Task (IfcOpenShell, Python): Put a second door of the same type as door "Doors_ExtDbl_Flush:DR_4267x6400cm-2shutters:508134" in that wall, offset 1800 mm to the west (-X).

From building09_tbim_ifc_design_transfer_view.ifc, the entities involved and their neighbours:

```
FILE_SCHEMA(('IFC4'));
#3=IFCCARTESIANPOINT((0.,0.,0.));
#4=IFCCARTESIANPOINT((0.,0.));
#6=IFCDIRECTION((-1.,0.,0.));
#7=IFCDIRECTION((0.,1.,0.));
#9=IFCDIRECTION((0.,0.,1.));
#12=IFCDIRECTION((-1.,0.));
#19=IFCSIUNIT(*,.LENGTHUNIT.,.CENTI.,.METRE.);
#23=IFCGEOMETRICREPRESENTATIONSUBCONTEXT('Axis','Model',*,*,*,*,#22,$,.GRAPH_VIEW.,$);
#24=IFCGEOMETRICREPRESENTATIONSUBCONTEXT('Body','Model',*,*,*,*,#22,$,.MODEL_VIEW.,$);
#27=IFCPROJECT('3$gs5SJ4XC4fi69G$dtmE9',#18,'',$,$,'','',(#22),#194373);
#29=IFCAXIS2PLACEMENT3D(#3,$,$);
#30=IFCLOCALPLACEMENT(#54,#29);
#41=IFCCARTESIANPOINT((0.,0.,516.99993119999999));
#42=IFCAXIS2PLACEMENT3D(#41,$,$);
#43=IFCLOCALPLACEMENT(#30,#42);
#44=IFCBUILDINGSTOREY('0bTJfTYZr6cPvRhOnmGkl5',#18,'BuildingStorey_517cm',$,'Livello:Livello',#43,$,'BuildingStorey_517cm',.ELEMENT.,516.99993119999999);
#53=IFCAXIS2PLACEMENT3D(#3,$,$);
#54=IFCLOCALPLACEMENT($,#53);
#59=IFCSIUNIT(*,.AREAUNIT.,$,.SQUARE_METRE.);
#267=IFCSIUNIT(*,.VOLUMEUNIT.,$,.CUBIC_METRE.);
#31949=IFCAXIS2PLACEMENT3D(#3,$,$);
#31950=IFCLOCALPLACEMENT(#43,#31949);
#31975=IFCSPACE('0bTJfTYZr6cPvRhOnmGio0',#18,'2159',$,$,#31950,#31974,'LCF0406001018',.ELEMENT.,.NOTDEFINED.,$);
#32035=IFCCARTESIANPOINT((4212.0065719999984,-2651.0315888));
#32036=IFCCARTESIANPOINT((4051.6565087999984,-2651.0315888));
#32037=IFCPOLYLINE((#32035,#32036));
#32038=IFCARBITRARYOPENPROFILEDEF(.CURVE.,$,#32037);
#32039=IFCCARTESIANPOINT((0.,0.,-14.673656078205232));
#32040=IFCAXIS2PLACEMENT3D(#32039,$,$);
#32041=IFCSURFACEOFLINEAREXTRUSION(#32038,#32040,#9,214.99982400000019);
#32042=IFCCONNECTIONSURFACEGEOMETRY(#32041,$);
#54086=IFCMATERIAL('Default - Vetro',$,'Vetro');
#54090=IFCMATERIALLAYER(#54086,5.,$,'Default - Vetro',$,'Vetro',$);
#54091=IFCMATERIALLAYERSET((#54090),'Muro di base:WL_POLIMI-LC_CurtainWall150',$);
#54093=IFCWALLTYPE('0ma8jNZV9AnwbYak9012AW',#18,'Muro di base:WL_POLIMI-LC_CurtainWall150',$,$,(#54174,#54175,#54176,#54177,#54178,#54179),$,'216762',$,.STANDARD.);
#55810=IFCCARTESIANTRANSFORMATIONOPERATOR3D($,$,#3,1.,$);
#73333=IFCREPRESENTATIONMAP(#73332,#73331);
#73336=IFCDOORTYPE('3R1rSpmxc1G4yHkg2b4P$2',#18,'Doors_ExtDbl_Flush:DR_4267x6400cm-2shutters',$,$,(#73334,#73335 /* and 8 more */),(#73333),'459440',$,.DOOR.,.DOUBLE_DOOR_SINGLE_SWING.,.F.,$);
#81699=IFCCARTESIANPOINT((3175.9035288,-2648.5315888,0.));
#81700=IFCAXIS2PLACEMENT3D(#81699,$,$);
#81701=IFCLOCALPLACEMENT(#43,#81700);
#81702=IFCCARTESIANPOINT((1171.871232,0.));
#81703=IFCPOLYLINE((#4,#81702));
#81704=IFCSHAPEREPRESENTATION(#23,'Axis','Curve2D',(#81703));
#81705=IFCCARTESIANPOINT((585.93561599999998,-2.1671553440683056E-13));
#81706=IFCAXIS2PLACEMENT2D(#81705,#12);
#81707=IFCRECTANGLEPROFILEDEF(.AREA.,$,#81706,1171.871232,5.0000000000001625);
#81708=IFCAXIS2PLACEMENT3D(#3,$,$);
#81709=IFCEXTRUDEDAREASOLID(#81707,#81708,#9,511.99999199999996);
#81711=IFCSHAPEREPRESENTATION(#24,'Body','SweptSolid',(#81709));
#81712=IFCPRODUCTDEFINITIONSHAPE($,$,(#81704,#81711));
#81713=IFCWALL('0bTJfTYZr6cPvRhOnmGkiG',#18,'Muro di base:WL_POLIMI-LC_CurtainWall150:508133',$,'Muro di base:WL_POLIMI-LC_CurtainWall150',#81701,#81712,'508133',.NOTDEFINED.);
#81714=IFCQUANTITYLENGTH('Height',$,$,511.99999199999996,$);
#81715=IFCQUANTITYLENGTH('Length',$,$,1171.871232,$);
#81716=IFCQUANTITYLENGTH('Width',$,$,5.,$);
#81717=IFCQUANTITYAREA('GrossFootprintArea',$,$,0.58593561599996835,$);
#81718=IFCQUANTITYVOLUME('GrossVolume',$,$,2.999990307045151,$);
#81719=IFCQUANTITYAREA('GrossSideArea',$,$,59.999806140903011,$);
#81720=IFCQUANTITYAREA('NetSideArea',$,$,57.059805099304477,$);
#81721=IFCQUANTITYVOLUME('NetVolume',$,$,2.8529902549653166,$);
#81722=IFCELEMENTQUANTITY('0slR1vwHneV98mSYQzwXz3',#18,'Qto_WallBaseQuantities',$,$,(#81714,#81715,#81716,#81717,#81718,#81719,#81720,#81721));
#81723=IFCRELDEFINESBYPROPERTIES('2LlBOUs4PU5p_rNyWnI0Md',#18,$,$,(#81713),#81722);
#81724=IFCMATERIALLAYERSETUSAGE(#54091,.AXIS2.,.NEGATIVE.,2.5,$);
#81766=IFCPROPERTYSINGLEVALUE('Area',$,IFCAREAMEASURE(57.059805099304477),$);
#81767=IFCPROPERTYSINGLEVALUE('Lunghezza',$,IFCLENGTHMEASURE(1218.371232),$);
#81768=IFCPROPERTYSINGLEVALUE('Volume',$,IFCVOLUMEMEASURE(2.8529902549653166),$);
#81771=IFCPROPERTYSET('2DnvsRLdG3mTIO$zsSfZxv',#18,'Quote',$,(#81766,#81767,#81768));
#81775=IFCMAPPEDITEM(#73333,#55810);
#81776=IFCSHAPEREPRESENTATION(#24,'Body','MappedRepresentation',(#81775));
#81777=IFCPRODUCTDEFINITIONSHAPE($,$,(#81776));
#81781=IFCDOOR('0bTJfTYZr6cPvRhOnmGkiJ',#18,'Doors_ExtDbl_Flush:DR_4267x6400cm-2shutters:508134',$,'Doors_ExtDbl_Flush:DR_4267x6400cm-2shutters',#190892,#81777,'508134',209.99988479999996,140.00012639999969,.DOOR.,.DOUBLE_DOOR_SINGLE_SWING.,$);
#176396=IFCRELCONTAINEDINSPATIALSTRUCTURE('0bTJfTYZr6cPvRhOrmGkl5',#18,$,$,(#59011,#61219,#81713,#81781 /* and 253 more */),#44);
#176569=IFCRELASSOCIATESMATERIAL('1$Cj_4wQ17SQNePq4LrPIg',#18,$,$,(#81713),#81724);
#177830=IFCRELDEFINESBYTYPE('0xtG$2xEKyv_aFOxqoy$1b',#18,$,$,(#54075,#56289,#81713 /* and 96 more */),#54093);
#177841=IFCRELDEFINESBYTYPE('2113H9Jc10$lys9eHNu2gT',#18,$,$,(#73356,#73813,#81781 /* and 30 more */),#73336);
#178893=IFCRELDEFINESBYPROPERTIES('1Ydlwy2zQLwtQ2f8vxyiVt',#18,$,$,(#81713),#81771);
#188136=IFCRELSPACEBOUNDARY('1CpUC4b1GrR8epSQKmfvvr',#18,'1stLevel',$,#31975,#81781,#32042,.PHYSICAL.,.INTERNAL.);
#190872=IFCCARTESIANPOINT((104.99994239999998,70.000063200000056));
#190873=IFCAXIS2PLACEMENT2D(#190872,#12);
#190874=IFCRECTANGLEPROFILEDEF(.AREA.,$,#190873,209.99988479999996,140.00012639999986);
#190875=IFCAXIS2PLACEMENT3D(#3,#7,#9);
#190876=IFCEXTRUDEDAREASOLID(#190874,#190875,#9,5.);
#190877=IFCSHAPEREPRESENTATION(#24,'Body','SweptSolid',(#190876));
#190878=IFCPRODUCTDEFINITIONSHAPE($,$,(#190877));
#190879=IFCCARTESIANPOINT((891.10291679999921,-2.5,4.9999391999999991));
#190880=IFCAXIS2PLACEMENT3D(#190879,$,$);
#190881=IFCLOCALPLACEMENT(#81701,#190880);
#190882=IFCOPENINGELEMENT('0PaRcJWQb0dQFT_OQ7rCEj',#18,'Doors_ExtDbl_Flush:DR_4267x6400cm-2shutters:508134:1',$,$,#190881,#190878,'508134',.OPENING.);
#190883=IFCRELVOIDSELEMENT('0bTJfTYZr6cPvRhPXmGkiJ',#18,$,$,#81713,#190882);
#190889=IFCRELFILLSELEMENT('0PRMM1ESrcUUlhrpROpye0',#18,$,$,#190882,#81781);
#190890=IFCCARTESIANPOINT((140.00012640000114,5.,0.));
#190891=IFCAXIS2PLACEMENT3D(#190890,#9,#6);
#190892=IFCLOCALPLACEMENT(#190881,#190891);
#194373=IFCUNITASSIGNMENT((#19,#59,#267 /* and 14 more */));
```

```python
import numpy as np
import ifcopenshell
import ifcopenshell.api.feature
import ifcopenshell.api.geometry
import ifcopenshell.api.pset
import ifcopenshell.api.root
import ifcopenshell.geom
import ifcopenshell.util.element
import ifcopenshell.util.placement
import ifcopenshell.util.shape
import ifcopenshell.util.unit

model = ifcopenshell.open("building09_tbim_ifc_design_transfer_view.ifc")
unit_scale = ifcopenshell.util.unit.calculate_unit_scale(model)
area_scale = ifcopenshell.util.unit.calculate_unit_scale(model, "AREAUNIT")
volume_scale = ifcopenshell.util.unit.calculate_unit_scale(model, "VOLUMEUNIT")
settings = ifcopenshell.geom.settings()


def volume(element):
    """Net volume in cubic metres, openings subtracted."""
    shape = ifcopenshell.geom.create_shape(settings, element)
    return ifcopenshell.util.shape.get_volume(shape.geometry)


def reuse_history(source, copy):
    """copy_class also copies each property set's owner history, people and application; keep the originals."""
    for rel in copy.IsDefinedBy:
        if rel.is_a("IfcRelDefinesByProperties") and (history := rel.RelatingPropertyDefinition.OwnerHistory):
            rel.RelatingPropertyDefinition.OwnerHistory = source.OwnerHistory
            ifcopenshell.util.element.remove_deep2(model, history)


door = model.by_guid("0bTJfTYZr6cPvRhOnmGkiJ")
opening = door.FillsVoids[0].RelatingOpeningElement
wall = opening.VoidsElements[0].RelatingBuildingElement
before = volume(wall)
shift = ifcopenshell.util.placement.get_local_placement(wall.ObjectPlacement)[:3, 0] * -1.8 / unit_scale

# copy_class copies the void relationship, type, container and properties, but no geometry.
new_opening = ifcopenshell.api.root.copy_class(model, product=opening)
new_opening.Representation = ifcopenshell.util.element.copy_deep(
    model, opening.Representation, exclude=["IfcGeometricRepresentationContext", "IfcRepresentationMap"]
)
new_opening.Name = "Doors_ExtDbl_Flush:DR_4267x6400cm-2shutters"
new_opening.Tag = None
reuse_history(opening, new_opening)
new_door = ifcopenshell.api.root.copy_class(model, product=door)
new_door.Representation = ifcopenshell.util.element.copy_deep(
    model, door.Representation, exclude=["IfcGeometricRepresentationContext", "IfcRepresentationMap"]
)
new_door.Name = "Doors_ExtDbl_Flush:DR_4267x6400cm-2shutters"
new_door.Tag = None
reuse_history(door, new_door)
ifcopenshell.api.feature.add_filling(model, opening=new_opening, element=new_door)

for old, new in ((opening, new_opening), (door, new_door)):
    matrix = ifcopenshell.util.placement.get_local_placement(old.ObjectPlacement)
    matrix[:3, 3] += shift
    ifcopenshell.api.geometry.edit_object_placement(model, product=new, matrix=matrix, is_si=False)

# The copied space boundaries still share their surfaces with the original.
for rel in new_door.ProvidesBoundaries:
    if rel.ConnectionGeometry:
        rel.ConnectionGeometry = ifcopenshell.util.element.copy_deep(model, rel.ConnectionGeometry)

# Space boundary surfaces are stored in each space's coordinates; move them too.
for rel in new_door.ProvidesBoundaries:
    if not rel.ConnectionGeometry:
        continue
    surface = rel.ConnectionGeometry.SurfaceOnRelatingElement
    space_matrix = ifcopenshell.util.placement.get_local_placement(rel.RelatingSpace.ObjectPlacement)
    point = np.array(surface.Position.Location.Coordinates) + space_matrix[:3, :3].T @ shift
    surface.Position = model.createIfcAxis2Placement3D(
        model.createIfcCartesianPoint(point.tolist()), surface.Position.Axis, surface.Position.RefDirection
    )

after = volume(wall)
thickness = 0.05  # wall thickness in metres

# Update the wall's stored quantities.
qto = model.by_id(ifcopenshell.util.element.get_pset(wall, "Qto_WallBaseQuantities", should_inherit=False)["id"])
ifcopenshell.api.pset.edit_qto(model, qto=qto, properties={
    "NetSideArea": after / thickness / area_scale,
    "NetVolume": after / volume_scale,
})
pset = model.by_id(ifcopenshell.util.element.get_pset(wall, "Quote", should_inherit=False)["id"])
ifcopenshell.api.pset.edit_pset(model, pset=pset, properties={
    "Area": model.create_entity("IfcAreaMeasure", after / thickness / area_scale),
    "Volume": model.create_entity("IfcVolumeMeasure", after / volume_scale),
})

print(f"wall volume {before:.3f} -> {after:.3f} m3")

model.write("building09_tbim_ifc_design_transfer_view_updated.ifc")
```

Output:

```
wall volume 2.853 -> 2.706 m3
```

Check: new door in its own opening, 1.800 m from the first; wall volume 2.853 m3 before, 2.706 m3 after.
